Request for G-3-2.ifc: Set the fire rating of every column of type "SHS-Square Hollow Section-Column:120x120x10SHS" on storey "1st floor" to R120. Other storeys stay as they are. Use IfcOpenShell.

First a look at what the model holds.

```python
import ifcopenshell
import ifcopenshell.util.element

model = ifcopenshell.open("G-3-2.ifc")
print(model.schema)
storey = next(s for s in model.by_type("IfcBuildingStorey") if s.Name == "1st floor")
columns = [e for e in ifcopenshell.util.element.get_decomposition(storey) if e.is_a("IfcColumn")]
seen = {}
for e in columns:
    element_type = ifcopenshell.util.element.get_type(e)
    key = (element_type.Name if element_type != e and element_type else None, ifcopenshell.util.element.get_pset(e, "Pset_ColumnCommon", "FireRating"))
    seen[key] = seen.get(key, 0) + 1
for (name, value), count in sorted(seen.items(), key=str):
    print(count, "x", name, "|", value)
```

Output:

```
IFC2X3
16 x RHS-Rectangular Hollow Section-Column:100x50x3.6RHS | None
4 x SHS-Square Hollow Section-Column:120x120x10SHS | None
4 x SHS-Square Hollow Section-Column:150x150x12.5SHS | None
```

```python
import ifcopenshell
import ifcopenshell.api.pset
import ifcopenshell.util.element

model = ifcopenshell.open("G-3-2.ifc")

storey = next(s for s in model.by_type("IfcBuildingStorey") if s.Name == "1st floor")
columns = [e for e in ifcopenshell.util.element.get_decomposition(storey) if e.is_a("IfcColumn")]

count = 0
for e in columns:
    element_type = ifcopenshell.util.element.get_type(e)
    if element_type in (None, e) or element_type.Name != "SHS-Square Hollow Section-Column:120x120x10SHS":
        continue
    # add_pset returns the element's existing set when there is one.
    pset = ifcopenshell.api.pset.add_pset(model, product=e, name="Pset_ColumnCommon")
    ifcopenshell.api.pset.edit_pset(model, pset=pset, properties={"FireRating": "R120"})
    count += 1

print(count, "columns updated")

model.write("G-3-2_updated.ifc")
```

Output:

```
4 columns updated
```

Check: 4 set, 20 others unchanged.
